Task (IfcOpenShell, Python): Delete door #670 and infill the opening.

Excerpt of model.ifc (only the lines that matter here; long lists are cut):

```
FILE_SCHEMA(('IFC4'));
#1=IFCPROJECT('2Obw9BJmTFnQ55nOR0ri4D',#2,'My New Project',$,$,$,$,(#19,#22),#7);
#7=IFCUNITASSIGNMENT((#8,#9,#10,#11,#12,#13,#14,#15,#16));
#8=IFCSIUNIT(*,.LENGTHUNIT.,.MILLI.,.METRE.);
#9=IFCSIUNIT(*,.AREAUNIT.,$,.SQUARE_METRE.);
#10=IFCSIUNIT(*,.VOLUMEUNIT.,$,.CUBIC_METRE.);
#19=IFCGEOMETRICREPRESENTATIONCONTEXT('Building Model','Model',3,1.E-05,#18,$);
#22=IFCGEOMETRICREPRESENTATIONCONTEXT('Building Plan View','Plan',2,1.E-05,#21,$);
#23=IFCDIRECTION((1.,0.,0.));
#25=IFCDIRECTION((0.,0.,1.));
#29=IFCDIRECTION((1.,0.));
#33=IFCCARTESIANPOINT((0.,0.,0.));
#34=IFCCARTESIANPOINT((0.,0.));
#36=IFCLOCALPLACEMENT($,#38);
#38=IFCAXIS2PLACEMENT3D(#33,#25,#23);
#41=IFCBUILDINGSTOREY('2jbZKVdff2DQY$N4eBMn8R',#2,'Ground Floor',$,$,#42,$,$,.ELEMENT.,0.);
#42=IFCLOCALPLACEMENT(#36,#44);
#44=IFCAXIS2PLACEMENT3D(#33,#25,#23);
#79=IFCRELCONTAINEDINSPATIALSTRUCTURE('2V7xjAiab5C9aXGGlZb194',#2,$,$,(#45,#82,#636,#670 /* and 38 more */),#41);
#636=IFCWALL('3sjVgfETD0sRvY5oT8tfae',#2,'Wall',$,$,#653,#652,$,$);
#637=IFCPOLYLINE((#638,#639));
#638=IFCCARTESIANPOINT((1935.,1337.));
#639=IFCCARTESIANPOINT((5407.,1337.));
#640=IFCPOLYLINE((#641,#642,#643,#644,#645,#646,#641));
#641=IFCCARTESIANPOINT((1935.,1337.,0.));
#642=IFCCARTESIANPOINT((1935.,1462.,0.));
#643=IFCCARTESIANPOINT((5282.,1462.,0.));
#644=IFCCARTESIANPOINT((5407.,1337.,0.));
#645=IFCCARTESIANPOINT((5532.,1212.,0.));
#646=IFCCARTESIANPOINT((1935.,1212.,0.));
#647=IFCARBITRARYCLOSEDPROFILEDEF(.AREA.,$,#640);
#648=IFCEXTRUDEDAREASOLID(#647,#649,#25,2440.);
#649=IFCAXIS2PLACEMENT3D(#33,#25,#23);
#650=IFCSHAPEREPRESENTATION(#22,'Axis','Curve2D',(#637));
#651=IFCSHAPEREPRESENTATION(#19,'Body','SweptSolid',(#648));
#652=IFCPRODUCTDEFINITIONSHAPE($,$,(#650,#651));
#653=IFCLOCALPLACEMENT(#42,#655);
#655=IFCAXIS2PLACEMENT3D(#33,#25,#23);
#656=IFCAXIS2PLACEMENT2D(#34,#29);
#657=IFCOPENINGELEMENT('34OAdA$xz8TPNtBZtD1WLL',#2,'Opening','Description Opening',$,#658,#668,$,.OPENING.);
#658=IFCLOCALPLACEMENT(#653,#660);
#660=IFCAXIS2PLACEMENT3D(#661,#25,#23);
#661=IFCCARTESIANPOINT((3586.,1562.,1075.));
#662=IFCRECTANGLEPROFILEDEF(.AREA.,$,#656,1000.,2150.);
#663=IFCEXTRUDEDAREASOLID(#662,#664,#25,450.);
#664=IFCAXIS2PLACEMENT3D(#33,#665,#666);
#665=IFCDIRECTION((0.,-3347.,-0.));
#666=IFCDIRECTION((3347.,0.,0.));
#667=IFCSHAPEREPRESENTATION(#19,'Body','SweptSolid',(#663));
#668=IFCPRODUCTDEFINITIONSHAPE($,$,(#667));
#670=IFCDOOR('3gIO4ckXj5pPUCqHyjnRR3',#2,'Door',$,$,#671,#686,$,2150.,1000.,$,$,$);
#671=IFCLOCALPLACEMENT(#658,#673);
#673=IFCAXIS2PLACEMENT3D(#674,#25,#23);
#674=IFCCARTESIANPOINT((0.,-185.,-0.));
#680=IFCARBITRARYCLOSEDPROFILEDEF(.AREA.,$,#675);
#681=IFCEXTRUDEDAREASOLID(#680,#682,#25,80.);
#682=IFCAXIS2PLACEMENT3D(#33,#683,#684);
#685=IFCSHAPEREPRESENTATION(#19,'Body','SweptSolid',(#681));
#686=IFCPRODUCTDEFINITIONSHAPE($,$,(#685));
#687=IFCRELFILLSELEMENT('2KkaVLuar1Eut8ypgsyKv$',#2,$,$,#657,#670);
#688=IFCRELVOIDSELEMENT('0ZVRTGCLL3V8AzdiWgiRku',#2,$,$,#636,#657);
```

```python
import ifcopenshell
import ifcopenshell.api.feature
import ifcopenshell.api.root
import ifcopenshell.geom
import ifcopenshell.util.shape

model = ifcopenshell.open("model.ifc")
settings = ifcopenshell.geom.settings()


def volume(element):
    """Net volume in cubic metres, openings subtracted."""
    shape = ifcopenshell.geom.create_shape(settings, element)
    return ifcopenshell.util.shape.get_volume(shape.geometry)


door = model.by_guid("3gIO4ckXj5pPUCqHyjnRR3")
opening = door.FillsVoids[0].RelatingOpeningElement
wall = opening.VoidsElements[0].RelatingBuildingElement
before = volume(wall)

ifcopenshell.api.root.remove_product(model, product=door)
ifcopenshell.api.feature.remove_feature(model, feature=opening)

after = volume(wall)

print(f"wall volume {before:.3f} -> {after:.3f} m3")

model.write("model-out.ifc")
```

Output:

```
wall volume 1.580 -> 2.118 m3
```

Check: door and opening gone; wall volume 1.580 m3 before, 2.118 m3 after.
